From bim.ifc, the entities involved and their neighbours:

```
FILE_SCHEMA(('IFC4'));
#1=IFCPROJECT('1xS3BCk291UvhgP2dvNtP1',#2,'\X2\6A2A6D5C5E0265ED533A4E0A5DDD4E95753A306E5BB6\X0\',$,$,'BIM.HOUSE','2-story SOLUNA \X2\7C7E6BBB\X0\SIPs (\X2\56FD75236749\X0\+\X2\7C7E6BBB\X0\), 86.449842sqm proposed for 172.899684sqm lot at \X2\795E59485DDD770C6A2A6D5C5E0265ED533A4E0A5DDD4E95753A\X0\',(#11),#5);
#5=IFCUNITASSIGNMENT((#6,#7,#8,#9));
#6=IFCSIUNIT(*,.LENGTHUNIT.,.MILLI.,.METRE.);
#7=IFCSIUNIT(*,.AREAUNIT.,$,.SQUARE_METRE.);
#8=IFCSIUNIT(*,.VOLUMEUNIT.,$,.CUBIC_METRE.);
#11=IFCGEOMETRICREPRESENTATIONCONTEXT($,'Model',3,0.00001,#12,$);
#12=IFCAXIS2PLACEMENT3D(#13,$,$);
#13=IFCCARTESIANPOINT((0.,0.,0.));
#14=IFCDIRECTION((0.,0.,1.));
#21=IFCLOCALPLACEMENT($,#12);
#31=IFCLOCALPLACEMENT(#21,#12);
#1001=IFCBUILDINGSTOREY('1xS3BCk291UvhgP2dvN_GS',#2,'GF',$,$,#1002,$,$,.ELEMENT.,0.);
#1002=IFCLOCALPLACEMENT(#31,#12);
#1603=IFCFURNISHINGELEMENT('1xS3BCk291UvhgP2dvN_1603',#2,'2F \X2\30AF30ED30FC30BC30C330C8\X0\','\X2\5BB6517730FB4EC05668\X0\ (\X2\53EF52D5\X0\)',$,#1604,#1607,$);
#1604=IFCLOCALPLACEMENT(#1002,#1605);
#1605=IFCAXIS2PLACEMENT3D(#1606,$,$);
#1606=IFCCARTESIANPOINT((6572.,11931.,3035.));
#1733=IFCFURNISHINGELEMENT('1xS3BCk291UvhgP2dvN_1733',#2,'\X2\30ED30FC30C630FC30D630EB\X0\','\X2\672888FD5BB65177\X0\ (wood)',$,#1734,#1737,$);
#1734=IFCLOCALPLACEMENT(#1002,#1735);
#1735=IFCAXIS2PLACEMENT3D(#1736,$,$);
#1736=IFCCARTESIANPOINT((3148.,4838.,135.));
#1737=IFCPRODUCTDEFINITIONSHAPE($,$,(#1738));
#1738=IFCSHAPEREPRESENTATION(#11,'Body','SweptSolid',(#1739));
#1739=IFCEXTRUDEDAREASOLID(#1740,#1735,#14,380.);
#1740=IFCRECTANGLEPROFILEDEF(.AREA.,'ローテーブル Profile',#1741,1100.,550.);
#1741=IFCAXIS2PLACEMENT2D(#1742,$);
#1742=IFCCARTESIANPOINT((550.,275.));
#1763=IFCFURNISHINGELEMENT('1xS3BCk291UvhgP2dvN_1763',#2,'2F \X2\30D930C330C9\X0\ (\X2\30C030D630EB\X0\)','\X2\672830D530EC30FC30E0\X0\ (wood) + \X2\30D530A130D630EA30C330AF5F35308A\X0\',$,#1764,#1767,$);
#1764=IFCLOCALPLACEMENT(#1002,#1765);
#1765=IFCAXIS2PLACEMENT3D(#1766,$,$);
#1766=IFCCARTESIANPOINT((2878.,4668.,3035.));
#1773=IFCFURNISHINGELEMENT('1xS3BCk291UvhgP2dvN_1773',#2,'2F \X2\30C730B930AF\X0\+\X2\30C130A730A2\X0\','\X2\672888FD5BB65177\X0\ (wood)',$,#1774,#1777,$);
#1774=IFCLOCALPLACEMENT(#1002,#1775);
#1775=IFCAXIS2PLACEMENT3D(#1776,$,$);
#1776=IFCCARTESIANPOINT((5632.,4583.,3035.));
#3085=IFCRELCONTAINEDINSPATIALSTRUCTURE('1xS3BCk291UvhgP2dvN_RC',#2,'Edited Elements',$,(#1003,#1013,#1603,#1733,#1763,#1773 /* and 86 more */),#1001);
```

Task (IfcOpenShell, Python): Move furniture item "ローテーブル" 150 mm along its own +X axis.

```python
import ifcopenshell
import ifcopenshell.api.geometry
import ifcopenshell.util.placement
import ifcopenshell.util.unit

model = ifcopenshell.open("bim.ifc")
unit_scale = ifcopenshell.util.unit.calculate_unit_scale(model)

item = model.by_id(1733)
matrix = ifcopenshell.util.placement.get_local_placement(item.ObjectPlacement)
matrix[:3, 3] += matrix[:3, 0] * 0.15 / unit_scale
ifcopenshell.api.geometry.edit_object_placement(model, product=item, matrix=matrix, is_si=False)

print(ifcopenshell.util.placement.get_local_placement(item.ObjectPlacement).round(3) + 0.0)

model.write("bim-out.ifc")
```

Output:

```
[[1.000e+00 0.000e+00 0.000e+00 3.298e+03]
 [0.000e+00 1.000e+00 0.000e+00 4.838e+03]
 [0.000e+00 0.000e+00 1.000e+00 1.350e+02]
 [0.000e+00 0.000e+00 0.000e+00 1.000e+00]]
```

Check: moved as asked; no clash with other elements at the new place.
